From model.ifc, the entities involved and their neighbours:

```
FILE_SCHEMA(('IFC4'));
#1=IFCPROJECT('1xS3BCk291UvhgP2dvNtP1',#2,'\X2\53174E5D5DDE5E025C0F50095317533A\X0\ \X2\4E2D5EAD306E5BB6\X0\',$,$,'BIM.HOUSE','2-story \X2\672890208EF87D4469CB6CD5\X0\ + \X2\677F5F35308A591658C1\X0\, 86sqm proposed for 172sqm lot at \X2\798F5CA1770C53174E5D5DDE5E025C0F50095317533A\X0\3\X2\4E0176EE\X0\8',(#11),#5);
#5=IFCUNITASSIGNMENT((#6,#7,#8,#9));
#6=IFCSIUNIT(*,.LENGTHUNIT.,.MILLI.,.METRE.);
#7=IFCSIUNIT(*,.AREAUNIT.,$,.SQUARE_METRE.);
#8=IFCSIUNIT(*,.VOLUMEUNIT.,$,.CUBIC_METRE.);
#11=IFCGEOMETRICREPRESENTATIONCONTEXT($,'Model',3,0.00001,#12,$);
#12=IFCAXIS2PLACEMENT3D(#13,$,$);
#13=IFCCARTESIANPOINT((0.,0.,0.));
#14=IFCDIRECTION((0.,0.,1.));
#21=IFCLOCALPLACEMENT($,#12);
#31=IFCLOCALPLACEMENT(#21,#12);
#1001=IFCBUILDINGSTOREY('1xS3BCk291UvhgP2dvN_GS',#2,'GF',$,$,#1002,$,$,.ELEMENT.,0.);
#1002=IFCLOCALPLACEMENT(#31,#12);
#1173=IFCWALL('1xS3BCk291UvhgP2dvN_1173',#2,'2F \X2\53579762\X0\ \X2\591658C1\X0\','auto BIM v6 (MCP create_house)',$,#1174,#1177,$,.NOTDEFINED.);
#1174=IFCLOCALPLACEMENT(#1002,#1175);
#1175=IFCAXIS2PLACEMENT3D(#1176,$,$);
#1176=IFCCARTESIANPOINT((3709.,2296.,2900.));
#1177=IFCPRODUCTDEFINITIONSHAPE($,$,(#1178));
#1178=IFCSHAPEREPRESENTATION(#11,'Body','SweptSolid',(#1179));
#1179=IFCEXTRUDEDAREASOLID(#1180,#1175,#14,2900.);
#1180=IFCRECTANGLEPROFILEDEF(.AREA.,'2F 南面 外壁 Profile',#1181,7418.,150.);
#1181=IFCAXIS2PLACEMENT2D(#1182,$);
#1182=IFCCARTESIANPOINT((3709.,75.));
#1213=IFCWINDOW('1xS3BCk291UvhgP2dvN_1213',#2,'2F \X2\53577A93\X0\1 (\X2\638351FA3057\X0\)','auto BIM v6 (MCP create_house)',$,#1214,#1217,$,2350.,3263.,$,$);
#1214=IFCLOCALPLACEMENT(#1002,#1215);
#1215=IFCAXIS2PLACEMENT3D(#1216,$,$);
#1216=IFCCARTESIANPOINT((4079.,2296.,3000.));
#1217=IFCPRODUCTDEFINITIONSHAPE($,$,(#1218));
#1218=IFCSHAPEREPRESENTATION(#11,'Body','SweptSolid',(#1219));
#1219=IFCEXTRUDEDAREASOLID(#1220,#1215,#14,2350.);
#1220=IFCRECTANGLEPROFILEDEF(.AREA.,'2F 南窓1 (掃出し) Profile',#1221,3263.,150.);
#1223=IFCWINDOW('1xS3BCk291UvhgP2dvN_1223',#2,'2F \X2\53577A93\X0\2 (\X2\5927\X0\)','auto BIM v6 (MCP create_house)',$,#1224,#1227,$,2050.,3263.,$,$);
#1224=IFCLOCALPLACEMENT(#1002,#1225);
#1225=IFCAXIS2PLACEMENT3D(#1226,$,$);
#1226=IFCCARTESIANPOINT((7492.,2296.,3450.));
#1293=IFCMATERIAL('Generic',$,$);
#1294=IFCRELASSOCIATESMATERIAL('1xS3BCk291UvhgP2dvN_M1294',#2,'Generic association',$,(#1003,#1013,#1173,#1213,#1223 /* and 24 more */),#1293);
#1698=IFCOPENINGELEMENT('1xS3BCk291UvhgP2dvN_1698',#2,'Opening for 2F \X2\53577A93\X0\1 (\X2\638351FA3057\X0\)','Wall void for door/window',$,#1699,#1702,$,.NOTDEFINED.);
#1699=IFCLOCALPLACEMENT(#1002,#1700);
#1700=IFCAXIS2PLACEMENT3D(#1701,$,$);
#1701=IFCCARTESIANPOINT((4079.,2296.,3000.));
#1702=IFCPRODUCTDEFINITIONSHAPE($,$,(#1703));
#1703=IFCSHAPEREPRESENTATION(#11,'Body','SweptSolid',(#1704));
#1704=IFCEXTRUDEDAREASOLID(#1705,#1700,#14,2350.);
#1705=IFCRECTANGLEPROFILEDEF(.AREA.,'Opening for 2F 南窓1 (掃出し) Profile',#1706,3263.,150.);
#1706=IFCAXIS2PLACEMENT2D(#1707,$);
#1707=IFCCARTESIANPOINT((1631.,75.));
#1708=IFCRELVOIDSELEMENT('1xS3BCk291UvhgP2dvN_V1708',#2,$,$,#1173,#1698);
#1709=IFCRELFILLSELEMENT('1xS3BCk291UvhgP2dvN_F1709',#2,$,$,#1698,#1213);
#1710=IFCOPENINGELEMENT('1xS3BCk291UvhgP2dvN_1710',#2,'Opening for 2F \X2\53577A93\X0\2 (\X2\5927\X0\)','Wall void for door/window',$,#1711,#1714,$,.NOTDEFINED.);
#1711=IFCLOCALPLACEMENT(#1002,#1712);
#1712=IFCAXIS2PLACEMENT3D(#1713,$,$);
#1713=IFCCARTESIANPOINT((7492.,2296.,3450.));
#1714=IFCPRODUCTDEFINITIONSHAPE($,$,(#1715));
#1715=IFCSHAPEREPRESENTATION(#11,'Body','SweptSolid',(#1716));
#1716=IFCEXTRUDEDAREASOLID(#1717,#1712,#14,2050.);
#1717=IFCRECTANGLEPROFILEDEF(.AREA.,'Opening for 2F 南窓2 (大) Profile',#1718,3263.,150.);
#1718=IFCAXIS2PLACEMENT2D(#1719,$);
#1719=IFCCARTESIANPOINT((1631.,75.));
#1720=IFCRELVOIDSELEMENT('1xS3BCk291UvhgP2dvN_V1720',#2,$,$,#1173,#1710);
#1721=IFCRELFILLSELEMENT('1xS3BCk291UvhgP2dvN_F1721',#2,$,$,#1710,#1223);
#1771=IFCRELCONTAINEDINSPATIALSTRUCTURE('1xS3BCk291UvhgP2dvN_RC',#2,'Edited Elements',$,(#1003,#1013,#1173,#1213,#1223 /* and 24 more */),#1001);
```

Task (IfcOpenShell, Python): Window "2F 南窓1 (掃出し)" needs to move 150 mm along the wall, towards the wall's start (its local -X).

```python
import ifcopenshell
import ifcopenshell.api.geometry
import ifcopenshell.util.placement
import ifcopenshell.util.unit

model = ifcopenshell.open("model.ifc")
unit_scale = ifcopenshell.util.unit.calculate_unit_scale(model)

window = model.by_guid("1xS3BCk291UvhgP2dvN_1213")
opening = window.FillsVoids[0].RelatingOpeningElement
wall = opening.VoidsElements[0].RelatingBuildingElement

wall_matrix = ifcopenshell.util.placement.get_local_placement(wall.ObjectPlacement)
shift = wall_matrix[:3, 0] * -0.15 / unit_scale
before = ifcopenshell.util.placement.get_local_placement(window.ObjectPlacement)[:3, 3].copy()

# The window is not placed relative to its opening, so move both.
for product in (opening, window):
    matrix = ifcopenshell.util.placement.get_local_placement(product.ObjectPlacement)
    matrix[:3, 3] += shift
    ifcopenshell.api.geometry.edit_object_placement(model, product=product, matrix=matrix, is_si=False)

after = ifcopenshell.util.placement.get_local_placement(window.ObjectPlacement)[:3, 3]
print("window moved by", (after - before).round(3) + 0.0)

model.write("model_rev.ifc")
```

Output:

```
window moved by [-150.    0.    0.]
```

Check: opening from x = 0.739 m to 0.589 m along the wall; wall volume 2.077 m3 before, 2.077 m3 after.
